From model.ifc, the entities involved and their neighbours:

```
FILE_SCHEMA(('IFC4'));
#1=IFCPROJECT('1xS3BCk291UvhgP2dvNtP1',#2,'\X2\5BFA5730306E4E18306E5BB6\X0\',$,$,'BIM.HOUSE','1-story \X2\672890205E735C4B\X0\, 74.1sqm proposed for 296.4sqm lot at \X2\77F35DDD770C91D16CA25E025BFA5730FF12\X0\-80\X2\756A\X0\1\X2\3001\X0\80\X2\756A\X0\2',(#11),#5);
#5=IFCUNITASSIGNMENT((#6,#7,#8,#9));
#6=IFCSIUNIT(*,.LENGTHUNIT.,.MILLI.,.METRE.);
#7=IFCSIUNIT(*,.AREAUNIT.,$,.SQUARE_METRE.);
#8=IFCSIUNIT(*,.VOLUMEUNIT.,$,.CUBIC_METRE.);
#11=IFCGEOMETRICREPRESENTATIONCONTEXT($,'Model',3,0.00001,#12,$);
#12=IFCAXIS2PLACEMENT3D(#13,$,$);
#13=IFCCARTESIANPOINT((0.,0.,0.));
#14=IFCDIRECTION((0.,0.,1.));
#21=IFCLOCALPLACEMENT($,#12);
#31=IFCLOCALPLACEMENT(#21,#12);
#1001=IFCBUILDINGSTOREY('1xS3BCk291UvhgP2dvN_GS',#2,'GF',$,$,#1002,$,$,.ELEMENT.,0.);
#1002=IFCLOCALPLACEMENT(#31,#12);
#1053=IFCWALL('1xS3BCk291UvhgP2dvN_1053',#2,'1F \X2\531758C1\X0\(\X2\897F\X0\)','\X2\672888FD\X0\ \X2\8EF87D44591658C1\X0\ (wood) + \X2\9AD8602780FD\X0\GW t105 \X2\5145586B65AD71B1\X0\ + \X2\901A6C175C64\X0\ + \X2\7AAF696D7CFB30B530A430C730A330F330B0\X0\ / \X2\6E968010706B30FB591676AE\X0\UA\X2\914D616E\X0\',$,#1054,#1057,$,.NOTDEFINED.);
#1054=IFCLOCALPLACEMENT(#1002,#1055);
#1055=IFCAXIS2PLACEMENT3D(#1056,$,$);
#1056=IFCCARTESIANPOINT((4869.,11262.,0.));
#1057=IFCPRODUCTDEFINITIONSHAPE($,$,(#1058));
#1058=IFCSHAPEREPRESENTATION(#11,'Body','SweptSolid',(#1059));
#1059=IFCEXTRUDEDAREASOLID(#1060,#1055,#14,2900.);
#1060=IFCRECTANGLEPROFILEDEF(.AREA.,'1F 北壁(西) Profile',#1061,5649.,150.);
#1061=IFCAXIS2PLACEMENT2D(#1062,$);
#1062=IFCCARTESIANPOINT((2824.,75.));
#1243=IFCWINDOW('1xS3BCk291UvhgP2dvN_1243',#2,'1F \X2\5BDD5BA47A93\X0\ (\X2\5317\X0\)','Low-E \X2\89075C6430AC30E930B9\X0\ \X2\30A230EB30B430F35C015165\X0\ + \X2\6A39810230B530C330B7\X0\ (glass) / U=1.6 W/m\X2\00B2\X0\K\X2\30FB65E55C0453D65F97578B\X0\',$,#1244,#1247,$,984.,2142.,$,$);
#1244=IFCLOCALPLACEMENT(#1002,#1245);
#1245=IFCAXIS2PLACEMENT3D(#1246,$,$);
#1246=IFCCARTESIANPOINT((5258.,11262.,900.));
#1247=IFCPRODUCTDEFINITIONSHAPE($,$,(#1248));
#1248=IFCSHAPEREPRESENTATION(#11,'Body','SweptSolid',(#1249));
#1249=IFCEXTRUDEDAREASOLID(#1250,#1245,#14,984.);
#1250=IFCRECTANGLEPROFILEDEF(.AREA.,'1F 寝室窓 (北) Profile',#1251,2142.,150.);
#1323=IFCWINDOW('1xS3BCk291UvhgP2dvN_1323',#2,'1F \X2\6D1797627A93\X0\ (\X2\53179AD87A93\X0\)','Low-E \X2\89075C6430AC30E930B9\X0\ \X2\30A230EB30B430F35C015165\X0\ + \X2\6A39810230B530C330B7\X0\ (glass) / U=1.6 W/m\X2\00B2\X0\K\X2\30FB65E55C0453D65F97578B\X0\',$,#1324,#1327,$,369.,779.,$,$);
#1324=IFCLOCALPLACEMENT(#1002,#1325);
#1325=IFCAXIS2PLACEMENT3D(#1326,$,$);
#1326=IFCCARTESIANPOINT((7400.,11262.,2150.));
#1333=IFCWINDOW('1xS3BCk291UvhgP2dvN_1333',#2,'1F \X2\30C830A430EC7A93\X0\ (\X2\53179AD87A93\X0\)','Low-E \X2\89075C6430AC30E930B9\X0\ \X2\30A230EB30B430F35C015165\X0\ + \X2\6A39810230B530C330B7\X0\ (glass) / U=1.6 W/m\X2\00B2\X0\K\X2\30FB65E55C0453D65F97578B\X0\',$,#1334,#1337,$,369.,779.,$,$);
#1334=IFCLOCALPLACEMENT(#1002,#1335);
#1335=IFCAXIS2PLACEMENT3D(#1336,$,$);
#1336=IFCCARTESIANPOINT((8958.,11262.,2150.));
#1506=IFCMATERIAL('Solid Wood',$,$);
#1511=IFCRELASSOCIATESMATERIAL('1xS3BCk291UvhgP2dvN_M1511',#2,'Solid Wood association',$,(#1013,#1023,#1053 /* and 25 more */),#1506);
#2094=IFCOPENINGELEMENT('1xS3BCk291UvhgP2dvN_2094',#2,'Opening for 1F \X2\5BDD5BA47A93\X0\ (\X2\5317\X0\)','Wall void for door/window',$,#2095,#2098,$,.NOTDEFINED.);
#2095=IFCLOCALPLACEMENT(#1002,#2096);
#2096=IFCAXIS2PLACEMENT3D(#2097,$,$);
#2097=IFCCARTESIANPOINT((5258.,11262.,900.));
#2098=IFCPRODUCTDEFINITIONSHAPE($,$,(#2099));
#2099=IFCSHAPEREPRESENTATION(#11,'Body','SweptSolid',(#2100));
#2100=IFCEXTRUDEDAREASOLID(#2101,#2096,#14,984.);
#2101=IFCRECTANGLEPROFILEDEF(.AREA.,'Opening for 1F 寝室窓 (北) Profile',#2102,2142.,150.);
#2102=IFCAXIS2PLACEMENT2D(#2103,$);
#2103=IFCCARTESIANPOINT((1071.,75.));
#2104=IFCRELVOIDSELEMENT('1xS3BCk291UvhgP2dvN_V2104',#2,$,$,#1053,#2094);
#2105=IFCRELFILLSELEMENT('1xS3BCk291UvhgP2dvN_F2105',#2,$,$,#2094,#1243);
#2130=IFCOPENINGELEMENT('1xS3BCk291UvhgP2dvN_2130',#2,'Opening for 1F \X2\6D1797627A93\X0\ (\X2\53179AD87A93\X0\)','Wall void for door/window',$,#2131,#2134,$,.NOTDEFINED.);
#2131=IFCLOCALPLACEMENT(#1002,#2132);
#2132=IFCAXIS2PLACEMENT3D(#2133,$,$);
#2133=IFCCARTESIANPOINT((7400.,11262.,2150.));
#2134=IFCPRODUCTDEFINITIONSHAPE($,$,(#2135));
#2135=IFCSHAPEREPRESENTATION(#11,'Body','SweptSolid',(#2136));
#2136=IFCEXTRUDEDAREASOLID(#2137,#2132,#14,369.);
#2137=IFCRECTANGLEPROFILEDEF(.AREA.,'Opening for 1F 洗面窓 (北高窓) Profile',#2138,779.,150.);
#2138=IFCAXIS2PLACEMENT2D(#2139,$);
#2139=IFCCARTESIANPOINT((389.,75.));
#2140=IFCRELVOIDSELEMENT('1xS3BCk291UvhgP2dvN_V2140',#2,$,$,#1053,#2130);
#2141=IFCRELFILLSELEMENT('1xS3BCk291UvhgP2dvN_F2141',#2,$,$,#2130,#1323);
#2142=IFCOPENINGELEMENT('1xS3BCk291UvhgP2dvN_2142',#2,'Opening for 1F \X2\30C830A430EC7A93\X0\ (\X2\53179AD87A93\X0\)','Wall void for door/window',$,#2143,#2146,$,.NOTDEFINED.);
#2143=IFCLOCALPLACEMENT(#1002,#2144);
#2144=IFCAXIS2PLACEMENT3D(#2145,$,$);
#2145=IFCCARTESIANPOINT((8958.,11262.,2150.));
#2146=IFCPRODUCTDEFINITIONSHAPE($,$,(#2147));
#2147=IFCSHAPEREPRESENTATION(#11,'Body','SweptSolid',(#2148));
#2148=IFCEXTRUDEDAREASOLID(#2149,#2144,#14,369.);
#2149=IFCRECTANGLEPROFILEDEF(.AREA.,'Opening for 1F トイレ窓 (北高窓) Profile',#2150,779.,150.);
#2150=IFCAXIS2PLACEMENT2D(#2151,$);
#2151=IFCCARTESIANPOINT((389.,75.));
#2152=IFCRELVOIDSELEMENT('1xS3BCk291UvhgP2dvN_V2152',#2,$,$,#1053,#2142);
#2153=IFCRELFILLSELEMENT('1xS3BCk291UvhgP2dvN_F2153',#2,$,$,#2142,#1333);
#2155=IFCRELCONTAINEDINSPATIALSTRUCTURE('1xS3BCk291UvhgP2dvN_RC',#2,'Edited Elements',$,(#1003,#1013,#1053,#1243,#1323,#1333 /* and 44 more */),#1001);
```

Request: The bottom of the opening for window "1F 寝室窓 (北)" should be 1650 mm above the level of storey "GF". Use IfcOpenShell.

```python
import numpy as np
import ifcopenshell
import ifcopenshell.api.geometry
import ifcopenshell.geom
import ifcopenshell.util.element
import ifcopenshell.util.placement
import ifcopenshell.util.shape
import ifcopenshell.util.unit

model = ifcopenshell.open("model.ifc")
unit_scale = ifcopenshell.util.unit.calculate_unit_scale(model)

window = model.by_guid("1xS3BCk291UvhgP2dvN_1243")
opening = window.FillsVoids[0].RelatingOpeningElement
storey = ifcopenshell.util.element.get_container(window, ifc_class="IfcBuildingStorey")
level = ifcopenshell.util.placement.get_local_placement(storey.ObjectPlacement)[2, 3]

# The opening's origin need not be at the sill, so measure its lowest point.
shape = ifcopenshell.geom.create_shape(ifcopenshell.geom.settings(), opening)
bottom = ifcopenshell.util.shape.get_shape_bottom_elevation(shape, shape.geometry) / unit_scale
dz = level + 1.65 / unit_scale - bottom

shift = np.array([0.0, 0.0, dz])
# The window is not placed relative to its opening, so move both.
for product in (opening, window):
    matrix = ifcopenshell.util.placement.get_local_placement(product.ObjectPlacement)
    matrix[:3, 3] += shift
    ifcopenshell.api.geometry.edit_object_placement(model, product=product, matrix=matrix, is_si=False)

print(f"moved by {dz * unit_scale:+.3f} m")

model.write("model_rev.ifc")
```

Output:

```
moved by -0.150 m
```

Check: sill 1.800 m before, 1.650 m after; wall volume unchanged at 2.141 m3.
